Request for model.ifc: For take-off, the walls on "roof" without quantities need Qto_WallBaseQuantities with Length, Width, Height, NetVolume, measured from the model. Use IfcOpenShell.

First a look at what the model holds.

```python
import ifcopenshell
import ifcopenshell.util.element
import ifcopenshell.util.unit

model = ifcopenshell.open("model.ifc")
print(model.schema)
for unit_type in ("LENGTHUNIT", "AREAUNIT", "VOLUMEUNIT"):
    print(unit_type, ifcopenshell.util.unit.calculate_unit_scale(model, unit_type))
storey = next(s for s in model.by_type("IfcBuildingStorey") if s.Name == "roof")
walls = [e for e in ifcopenshell.util.element.get_decomposition(storey) if e.is_a("IfcWall")]
for e in sorted(walls, key=lambda e: e.id()):
    print(e.id(), e.is_a(), e.Name, list(ifcopenshell.util.element.get_psets(e, qtos_only=True)), sep=" | ")
```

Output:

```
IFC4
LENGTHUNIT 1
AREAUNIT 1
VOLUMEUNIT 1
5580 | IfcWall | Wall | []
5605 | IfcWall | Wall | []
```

```python
import ifcopenshell
import ifcopenshell.api.pset
import ifcopenshell.geom
import ifcopenshell.util.element
import ifcopenshell.util.shape
import ifcopenshell.util.unit

model = ifcopenshell.open("model.ifc")
unit_scale = ifcopenshell.util.unit.calculate_unit_scale(model)
volume_scale = ifcopenshell.util.unit.calculate_unit_scale(model, "VOLUMEUNIT")
settings = ifcopenshell.geom.settings()

storey = next(s for s in model.by_type("IfcBuildingStorey") if s.Name == "roof")
walls = [e for e in ifcopenshell.util.element.get_decomposition(storey) if e.is_a("IfcWall")]

for e in sorted(walls, key=lambda e: e.id()):
    if ifcopenshell.util.element.get_psets(e, qtos_only=True, should_inherit=False):
        continue
    # Geometry comes back in metres, in the element's own axes.
    shape = ifcopenshell.geom.create_shape(settings, e)
    values = {
        "Length": ifcopenshell.util.shape.get_x(shape.geometry) / unit_scale,
        "Width": ifcopenshell.util.shape.get_y(shape.geometry) / unit_scale,
        "Height": ifcopenshell.util.shape.get_z(shape.geometry) / unit_scale,
        "NetVolume": ifcopenshell.util.shape.get_volume(shape.geometry) / volume_scale,
    }
    qto = ifcopenshell.api.pset.add_qto(model, product=e, name="Qto_WallBaseQuantities")
    ifcopenshell.api.pset.edit_qto(model, qto=qto, properties=values)
    print(e.id(), {k: round(v, 3) for k, v in values.items()})

model.write("model_v2.ifc")
```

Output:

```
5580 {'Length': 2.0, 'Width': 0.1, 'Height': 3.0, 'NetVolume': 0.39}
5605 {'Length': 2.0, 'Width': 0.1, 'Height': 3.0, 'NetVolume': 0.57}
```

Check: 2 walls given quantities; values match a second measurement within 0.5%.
